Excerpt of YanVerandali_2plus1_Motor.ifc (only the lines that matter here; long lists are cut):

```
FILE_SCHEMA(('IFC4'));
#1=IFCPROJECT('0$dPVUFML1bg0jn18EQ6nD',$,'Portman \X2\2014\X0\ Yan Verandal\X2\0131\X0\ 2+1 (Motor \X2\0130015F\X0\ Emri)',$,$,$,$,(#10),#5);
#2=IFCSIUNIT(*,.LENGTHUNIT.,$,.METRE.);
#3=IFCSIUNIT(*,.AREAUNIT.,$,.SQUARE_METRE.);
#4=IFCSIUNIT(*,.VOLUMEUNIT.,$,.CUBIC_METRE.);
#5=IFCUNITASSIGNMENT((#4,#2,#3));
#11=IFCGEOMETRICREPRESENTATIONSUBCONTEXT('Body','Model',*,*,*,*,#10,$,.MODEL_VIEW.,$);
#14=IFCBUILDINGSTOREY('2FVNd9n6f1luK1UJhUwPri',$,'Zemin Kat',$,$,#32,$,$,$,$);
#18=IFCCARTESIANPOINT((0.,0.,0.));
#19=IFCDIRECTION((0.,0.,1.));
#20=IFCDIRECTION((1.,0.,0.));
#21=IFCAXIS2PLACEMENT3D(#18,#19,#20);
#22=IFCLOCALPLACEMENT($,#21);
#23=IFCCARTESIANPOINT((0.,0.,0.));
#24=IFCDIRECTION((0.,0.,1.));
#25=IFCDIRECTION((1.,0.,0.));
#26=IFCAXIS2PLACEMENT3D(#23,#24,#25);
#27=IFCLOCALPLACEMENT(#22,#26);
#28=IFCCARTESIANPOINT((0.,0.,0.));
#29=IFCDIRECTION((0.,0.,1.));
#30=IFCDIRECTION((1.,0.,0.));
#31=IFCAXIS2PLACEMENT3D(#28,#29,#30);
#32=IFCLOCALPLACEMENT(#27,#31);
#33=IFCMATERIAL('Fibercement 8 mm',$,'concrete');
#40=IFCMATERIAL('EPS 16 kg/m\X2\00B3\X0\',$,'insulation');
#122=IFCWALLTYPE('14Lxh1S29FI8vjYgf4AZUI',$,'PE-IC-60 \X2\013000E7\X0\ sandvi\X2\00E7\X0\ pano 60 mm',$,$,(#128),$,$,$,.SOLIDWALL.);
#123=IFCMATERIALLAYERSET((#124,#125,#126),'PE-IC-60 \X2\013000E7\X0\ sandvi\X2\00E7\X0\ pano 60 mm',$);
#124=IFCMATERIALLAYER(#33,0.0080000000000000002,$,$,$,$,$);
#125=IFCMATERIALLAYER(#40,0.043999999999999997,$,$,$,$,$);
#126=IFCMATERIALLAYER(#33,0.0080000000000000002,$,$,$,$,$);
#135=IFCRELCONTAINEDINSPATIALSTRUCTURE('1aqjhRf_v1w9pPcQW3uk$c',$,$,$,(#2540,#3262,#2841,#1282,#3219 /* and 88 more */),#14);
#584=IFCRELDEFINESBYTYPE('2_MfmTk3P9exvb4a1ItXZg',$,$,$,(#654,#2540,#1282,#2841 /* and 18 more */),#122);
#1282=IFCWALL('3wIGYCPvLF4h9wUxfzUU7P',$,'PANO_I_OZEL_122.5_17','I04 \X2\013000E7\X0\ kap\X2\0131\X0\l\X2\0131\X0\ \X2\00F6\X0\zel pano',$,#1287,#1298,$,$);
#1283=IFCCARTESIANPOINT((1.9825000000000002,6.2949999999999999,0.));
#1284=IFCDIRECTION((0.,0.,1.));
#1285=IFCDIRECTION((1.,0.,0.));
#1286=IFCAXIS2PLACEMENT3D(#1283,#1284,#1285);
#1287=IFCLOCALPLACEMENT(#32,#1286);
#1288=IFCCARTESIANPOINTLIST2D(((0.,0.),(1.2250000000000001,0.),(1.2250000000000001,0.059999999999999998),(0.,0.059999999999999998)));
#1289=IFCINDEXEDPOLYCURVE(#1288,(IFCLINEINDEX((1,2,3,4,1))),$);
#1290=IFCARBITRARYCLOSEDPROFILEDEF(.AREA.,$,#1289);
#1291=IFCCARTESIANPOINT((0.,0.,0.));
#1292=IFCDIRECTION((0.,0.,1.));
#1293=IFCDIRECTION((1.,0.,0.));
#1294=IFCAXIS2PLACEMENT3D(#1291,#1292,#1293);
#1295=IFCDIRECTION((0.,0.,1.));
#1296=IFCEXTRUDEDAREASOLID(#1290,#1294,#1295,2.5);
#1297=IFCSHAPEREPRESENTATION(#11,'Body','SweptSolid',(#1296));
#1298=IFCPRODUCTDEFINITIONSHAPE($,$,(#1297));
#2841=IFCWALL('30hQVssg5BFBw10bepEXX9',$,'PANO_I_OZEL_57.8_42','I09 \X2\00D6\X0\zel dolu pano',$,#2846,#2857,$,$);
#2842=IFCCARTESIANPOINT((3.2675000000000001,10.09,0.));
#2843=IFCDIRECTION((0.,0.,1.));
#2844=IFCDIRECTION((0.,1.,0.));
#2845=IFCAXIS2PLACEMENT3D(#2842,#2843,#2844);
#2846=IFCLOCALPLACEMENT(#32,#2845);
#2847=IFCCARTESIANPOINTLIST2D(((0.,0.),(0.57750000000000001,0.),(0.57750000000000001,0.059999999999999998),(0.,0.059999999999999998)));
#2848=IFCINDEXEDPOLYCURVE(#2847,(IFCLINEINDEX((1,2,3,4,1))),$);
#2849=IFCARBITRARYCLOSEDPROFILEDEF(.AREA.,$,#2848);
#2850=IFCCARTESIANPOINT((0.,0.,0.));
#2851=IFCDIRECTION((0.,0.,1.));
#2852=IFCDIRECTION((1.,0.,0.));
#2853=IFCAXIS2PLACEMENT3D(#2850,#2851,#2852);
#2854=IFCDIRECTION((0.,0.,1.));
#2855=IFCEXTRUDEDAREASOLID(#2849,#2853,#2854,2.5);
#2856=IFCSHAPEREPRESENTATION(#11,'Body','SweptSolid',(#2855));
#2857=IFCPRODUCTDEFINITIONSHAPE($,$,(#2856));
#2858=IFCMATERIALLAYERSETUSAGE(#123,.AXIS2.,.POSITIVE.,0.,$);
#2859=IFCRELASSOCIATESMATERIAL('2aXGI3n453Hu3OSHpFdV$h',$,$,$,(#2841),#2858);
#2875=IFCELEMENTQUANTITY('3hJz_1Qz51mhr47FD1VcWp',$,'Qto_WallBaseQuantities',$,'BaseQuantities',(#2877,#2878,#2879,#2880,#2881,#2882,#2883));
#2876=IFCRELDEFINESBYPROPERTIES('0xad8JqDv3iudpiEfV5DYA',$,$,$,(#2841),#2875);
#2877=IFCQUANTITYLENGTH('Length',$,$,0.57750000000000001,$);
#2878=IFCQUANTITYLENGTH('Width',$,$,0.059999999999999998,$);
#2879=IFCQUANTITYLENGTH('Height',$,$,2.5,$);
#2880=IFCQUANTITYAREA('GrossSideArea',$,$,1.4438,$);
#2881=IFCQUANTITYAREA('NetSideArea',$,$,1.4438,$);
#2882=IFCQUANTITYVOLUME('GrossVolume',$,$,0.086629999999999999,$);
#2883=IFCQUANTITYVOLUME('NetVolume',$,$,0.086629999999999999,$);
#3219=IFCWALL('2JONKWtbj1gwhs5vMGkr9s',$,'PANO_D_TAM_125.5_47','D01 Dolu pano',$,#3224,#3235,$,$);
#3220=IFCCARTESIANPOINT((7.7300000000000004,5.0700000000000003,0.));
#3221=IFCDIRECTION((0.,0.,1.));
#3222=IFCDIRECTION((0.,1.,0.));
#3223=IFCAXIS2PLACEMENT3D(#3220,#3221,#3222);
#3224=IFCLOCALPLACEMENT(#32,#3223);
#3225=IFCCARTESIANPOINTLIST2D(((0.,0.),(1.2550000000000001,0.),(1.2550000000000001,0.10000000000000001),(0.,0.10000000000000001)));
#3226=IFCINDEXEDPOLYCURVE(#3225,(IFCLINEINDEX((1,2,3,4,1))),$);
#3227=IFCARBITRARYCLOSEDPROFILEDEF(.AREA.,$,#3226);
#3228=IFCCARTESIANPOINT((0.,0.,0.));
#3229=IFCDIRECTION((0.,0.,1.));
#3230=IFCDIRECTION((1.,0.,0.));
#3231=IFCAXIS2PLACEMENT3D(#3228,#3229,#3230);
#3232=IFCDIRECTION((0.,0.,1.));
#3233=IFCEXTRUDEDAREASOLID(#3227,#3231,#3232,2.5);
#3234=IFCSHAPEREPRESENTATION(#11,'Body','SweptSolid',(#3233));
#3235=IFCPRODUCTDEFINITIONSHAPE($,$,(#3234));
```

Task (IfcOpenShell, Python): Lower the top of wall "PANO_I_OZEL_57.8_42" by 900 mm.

```python
import ifcopenshell
import ifcopenshell.api.pset
import ifcopenshell.geom
import ifcopenshell.util.element
import ifcopenshell.util.representation
import ifcopenshell.util.shape
import ifcopenshell.util.unit

model = ifcopenshell.open("YanVerandali_2plus1_Motor.ifc")
unit_scale = ifcopenshell.util.unit.calculate_unit_scale(model)
area_scale = ifcopenshell.util.unit.calculate_unit_scale(model, "AREAUNIT")
volume_scale = ifcopenshell.util.unit.calculate_unit_scale(model, "VOLUMEUNIT")
settings = ifcopenshell.geom.settings()


def volume(element):
    """Net volume in cubic metres, openings subtracted."""
    shape = ifcopenshell.geom.create_shape(settings, element)
    return ifcopenshell.util.shape.get_volume(shape.geometry)


wall = model.by_id(2841)
before = volume(wall)

body = ifcopenshell.util.representation.get_representation(wall, "Model", "Body")
solid = body.Items[0]
old_height = solid.Depth
solid.Depth -= 0.9 / unit_scale
after = volume(wall)
thickness = 0.06  # wall thickness in metres

# Update the stored height, areas and volumes.
qto = model.by_id(ifcopenshell.util.element.get_pset(wall, "Qto_WallBaseQuantities", should_inherit=False)["id"])
ifcopenshell.api.pset.edit_qto(model, qto=qto, properties={
    "Height": solid.Depth,
    "GrossSideArea": ifcopenshell.util.element.get_pset(wall, "Qto_WallBaseQuantities", "GrossSideArea") * solid.Depth / old_height,
    "NetSideArea": after / thickness / area_scale,
    "GrossVolume": ifcopenshell.util.element.get_pset(wall, "Qto_WallBaseQuantities", "GrossVolume") * solid.Depth / old_height,
    "NetVolume": after / volume_scale,
})

print(f"height {old_height:g} -> {solid.Depth:g}, volume {before:.3f} -> {after:.3f} m3")

model.write("YanVerandali_2plus1_Motor_rev.ifc")
```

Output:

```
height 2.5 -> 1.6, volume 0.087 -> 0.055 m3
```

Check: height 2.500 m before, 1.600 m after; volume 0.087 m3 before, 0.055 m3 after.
